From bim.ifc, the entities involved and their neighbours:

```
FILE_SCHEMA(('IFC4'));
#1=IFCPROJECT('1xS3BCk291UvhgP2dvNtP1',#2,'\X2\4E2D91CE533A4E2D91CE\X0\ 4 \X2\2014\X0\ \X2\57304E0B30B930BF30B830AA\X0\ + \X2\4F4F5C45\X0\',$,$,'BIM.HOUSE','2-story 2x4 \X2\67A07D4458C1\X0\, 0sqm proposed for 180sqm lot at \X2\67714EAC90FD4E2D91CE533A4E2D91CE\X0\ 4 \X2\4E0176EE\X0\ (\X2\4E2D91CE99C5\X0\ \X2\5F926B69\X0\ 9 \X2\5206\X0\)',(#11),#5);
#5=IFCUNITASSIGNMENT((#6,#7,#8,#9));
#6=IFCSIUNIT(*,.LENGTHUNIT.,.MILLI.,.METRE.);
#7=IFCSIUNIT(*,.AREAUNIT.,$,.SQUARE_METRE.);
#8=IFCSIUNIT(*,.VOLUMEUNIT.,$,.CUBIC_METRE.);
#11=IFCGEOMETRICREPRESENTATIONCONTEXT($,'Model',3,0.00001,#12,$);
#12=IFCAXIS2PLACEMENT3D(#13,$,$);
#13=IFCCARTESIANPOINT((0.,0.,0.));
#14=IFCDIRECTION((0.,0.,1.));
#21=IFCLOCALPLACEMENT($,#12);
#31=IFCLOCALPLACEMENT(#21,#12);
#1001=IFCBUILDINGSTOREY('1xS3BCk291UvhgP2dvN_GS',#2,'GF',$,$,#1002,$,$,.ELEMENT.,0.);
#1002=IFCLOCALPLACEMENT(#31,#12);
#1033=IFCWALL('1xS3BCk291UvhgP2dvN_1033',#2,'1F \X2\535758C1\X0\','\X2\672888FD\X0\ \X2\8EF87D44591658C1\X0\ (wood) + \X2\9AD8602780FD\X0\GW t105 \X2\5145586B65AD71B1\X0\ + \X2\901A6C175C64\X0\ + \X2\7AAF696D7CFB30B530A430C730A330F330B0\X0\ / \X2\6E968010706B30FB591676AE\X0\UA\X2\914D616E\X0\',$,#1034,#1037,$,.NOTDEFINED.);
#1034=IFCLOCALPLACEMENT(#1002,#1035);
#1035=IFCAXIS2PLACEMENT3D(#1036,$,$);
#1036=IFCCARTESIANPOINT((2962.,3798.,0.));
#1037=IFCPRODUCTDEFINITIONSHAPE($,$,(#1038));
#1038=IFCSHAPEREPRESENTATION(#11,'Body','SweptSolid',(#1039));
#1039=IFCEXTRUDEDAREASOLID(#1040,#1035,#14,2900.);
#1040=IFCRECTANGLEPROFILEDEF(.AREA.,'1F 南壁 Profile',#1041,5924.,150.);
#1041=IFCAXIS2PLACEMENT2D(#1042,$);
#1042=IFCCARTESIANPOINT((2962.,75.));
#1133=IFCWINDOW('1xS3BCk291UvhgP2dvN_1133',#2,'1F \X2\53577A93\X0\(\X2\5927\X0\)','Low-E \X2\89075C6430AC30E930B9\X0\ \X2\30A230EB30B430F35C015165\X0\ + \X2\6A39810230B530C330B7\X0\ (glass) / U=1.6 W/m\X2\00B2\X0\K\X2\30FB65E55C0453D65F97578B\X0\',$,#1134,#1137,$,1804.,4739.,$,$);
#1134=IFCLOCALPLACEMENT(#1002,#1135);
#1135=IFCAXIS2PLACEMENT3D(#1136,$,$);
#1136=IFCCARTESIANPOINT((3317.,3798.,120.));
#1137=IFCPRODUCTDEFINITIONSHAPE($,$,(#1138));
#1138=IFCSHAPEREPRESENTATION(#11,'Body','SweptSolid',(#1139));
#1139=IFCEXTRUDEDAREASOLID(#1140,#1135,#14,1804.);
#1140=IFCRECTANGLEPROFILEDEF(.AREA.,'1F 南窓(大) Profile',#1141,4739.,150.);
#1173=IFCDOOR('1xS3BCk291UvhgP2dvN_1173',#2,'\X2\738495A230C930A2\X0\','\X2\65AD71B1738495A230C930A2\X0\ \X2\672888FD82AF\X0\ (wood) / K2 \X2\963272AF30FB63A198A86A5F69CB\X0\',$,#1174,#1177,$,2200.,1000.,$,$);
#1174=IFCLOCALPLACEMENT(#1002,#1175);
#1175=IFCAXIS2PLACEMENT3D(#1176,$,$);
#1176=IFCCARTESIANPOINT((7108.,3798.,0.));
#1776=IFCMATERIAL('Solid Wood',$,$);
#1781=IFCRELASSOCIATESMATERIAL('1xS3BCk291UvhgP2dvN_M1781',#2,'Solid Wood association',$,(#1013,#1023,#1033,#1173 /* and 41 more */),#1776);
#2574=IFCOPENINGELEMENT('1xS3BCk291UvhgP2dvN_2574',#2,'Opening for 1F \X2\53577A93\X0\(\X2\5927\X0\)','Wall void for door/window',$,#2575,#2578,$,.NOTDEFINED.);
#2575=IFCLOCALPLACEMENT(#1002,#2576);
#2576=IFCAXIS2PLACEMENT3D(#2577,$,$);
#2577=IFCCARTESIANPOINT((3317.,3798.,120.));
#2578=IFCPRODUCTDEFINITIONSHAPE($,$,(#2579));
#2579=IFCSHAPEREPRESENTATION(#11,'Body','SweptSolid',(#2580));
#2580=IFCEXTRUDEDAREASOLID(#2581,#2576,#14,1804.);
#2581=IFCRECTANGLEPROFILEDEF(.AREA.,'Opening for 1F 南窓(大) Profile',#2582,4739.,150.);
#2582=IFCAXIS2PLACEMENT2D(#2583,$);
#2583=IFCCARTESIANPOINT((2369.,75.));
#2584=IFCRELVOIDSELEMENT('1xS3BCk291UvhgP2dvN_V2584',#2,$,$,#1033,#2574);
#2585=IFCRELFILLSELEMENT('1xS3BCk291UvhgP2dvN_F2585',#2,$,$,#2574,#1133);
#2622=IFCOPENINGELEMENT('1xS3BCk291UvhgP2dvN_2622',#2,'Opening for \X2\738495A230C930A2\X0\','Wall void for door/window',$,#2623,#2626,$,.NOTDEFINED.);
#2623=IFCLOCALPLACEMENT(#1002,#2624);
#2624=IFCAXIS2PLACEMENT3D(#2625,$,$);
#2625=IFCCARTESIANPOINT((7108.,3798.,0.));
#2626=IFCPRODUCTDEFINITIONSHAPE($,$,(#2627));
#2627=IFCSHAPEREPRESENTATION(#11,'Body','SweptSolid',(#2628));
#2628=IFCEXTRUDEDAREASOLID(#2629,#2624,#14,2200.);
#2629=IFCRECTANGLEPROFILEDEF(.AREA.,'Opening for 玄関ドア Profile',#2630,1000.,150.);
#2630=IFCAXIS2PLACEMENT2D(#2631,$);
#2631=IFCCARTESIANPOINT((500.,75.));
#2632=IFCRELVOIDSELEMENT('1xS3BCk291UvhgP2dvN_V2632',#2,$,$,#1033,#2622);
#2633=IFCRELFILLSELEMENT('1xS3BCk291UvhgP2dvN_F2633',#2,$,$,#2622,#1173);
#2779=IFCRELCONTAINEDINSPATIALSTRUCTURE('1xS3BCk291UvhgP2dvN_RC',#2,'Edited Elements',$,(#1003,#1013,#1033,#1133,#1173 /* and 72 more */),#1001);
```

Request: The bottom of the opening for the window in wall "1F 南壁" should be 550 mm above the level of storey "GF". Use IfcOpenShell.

```python
import numpy as np
import ifcopenshell
import ifcopenshell.api.geometry
import ifcopenshell.geom
import ifcopenshell.util.element
import ifcopenshell.util.placement
import ifcopenshell.util.shape
import ifcopenshell.util.unit

model = ifcopenshell.open("bim.ifc")
unit_scale = ifcopenshell.util.unit.calculate_unit_scale(model)

window = model.by_guid("1xS3BCk291UvhgP2dvN_1133")
opening = window.FillsVoids[0].RelatingOpeningElement
storey = ifcopenshell.util.element.get_container(window, ifc_class="IfcBuildingStorey")
level = ifcopenshell.util.placement.get_local_placement(storey.ObjectPlacement)[2, 3]

# The opening's origin need not be at the sill, so measure its lowest point.
shape = ifcopenshell.geom.create_shape(ifcopenshell.geom.settings(), opening)
bottom = ifcopenshell.util.shape.get_shape_bottom_elevation(shape, shape.geometry) / unit_scale
dz = level + 550.0 - bottom

shift = np.array([0.0, 0.0, dz])
# The window is not placed relative to its opening, so move both.
for product in (opening, window):
    matrix = ifcopenshell.util.placement.get_local_placement(product.ObjectPlacement)
    matrix[:3, 3] += shift
    ifcopenshell.api.geometry.edit_object_placement(model, product=product, matrix=matrix, is_si=False)

print(f"moved by {dz * unit_scale:+.3f} m")

model.write("bim_rev.ifc")
```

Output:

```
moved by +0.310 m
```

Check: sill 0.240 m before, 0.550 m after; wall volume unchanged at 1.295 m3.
